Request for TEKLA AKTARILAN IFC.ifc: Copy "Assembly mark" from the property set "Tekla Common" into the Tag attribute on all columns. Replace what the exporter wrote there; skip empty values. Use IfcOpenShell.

First a look at what the model holds.

```python
import ifcopenshell
import ifcopenshell.util.element

model = ifcopenshell.open("TEKLA AKTARILAN IFC.ifc")
print(model.schema)
columns = model.by_type("IfcColumn")
print(len(columns), "columns")
for e in columns[:8]:
    source = ifcopenshell.util.element.get_pset(e, "Tekla Common", "Assembly mark")
    target = e.Tag
    print(e.id(), repr(source), repr(target), sep=" | ")
```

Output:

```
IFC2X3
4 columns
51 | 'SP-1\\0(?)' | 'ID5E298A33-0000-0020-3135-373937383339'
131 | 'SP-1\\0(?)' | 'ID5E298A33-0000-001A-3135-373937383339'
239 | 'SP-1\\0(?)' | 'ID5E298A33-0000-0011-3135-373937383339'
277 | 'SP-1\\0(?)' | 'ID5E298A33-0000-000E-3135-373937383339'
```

```python
import ifcopenshell
import ifcopenshell.util.element

model = ifcopenshell.open("TEKLA AKTARILAN IFC.ifc")

count = 0
for e in model.by_type("IfcColumn"):
    value = ifcopenshell.util.element.get_pset(e, "Tekla Common", "Assembly mark")
    current = e.Tag
    if not value or not value.strip() or current == value:
        continue
    e.Tag = value
    count += 1

print(count, "columns updated")

model.write("TEKLA AKTARILAN IFC_edited.ifc")
```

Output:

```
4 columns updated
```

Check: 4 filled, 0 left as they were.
